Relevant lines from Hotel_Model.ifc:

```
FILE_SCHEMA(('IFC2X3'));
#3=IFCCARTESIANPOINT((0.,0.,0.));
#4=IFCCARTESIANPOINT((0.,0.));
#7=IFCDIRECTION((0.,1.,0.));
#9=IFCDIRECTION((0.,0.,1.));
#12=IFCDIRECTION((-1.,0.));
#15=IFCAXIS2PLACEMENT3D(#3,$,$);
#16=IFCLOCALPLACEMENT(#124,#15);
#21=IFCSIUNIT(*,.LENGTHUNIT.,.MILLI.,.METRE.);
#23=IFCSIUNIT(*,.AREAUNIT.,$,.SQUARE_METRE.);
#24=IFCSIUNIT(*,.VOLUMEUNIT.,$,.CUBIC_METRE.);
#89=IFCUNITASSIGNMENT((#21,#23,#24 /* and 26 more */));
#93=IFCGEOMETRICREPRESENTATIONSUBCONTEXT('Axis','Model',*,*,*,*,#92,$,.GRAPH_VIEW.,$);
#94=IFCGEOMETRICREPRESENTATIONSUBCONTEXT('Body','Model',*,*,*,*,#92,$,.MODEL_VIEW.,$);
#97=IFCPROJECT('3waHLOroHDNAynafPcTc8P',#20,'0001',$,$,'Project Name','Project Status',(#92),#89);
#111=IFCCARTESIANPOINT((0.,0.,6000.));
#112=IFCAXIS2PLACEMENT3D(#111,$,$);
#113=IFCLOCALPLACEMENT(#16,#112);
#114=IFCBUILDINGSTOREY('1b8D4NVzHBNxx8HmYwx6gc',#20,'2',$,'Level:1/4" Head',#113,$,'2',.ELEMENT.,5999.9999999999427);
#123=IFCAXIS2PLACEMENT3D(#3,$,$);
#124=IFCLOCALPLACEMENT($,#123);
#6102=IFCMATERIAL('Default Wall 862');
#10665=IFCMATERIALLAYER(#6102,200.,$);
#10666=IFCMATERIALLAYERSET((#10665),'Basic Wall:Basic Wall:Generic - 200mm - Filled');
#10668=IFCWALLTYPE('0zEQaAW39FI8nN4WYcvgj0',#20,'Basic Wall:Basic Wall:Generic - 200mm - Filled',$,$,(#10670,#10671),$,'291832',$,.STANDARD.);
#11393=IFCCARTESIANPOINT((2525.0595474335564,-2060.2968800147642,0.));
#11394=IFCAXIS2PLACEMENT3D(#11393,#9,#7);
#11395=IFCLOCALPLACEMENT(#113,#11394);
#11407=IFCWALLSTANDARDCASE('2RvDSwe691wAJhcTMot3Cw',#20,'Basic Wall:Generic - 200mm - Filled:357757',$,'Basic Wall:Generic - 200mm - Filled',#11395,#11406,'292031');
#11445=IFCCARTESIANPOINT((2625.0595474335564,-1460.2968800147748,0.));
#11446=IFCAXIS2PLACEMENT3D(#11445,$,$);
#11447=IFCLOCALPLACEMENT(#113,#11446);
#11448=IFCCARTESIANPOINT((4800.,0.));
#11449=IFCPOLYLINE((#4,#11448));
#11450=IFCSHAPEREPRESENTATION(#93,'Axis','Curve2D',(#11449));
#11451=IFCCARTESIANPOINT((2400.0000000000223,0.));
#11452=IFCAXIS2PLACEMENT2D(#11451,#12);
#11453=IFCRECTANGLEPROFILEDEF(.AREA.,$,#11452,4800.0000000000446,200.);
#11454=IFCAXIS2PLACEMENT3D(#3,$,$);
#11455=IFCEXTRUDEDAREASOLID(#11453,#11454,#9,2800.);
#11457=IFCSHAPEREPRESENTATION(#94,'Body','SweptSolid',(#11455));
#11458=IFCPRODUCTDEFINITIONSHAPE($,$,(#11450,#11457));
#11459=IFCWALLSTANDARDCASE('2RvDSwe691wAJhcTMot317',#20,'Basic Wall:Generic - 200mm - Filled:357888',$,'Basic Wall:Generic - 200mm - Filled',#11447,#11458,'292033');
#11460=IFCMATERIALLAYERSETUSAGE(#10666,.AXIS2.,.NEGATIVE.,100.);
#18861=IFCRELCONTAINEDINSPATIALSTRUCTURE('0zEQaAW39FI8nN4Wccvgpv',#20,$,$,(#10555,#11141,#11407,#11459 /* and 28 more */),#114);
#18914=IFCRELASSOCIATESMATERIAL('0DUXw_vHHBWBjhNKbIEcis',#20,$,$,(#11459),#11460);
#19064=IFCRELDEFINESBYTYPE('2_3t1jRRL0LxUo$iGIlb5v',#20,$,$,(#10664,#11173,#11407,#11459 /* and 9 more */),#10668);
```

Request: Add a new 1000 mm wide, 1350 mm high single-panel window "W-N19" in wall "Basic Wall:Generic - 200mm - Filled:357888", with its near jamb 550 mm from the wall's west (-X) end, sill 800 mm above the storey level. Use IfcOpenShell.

```python
import numpy as np
import ifcopenshell
import ifcopenshell.api.feature
import ifcopenshell.api.geometry
import ifcopenshell.api.root
import ifcopenshell.api.spatial
import ifcopenshell.api.type
import ifcopenshell.geom
import ifcopenshell.util.element
import ifcopenshell.util.placement
import ifcopenshell.util.representation
import ifcopenshell.util.shape
import ifcopenshell.util.unit

model = ifcopenshell.open("Hotel_Model.ifc")
unit_scale = ifcopenshell.util.unit.calculate_unit_scale(model)
settings = ifcopenshell.geom.settings()


def volume(element):
    """Net volume in cubic metres, openings subtracted."""
    shape = ifcopenshell.geom.create_shape(settings, element)
    return ifcopenshell.util.shape.get_volume(shape.geometry)


wall = model.by_id(11459)
storey = ifcopenshell.util.element.get_container(wall, ifc_class="IfcBuildingStorey")
context = ifcopenshell.util.representation.get_context(model, "Model", "Body", "MODEL_VIEW")
before = volume(wall)

width, height, from_end, sill = 1, 1.35, 0.55, 0.8  # metres

# The wall runs along its own X axis, and the end named is its -X end.
wall_shape = ifcopenshell.geom.create_shape(settings, wall)
x, y, z = ifcopenshell.util.shape.get_vertices(wall_shape.geometry).T
start = x.min() + from_end
face, thickness = float(y.min()), float(y.max() - y.min())
wall_matrix = ifcopenshell.util.placement.get_local_placement(wall.ObjectPlacement)
level = ifcopenshell.util.placement.get_local_placement(storey.ObjectPlacement)[2, 3]


def in_wall(x, y):
    """Placement at x, y metres in the wall's axes, at sill height."""
    matrix = wall_matrix.copy()
    matrix[:, 3] = wall_matrix @ np.array([x / unit_scale, y / unit_scale, 0.0, 1.0])
    matrix[2, 3] = level + sill / unit_scale
    return matrix


# Opening: a box that overshoots both wall faces by 50 mm.
opening = ifcopenshell.api.root.create_entity(model, ifc_class="IfcOpeningElement")
box = ifcopenshell.api.geometry.add_wall_representation(
    model, context=context, length=width, height=height, thickness=thickness + 0.1
)
ifcopenshell.api.geometry.assign_representation(model, product=opening, representation=box)
ifcopenshell.api.geometry.edit_object_placement(model, product=opening, matrix=in_wall(start, face - 0.05), is_si=False)
ifcopenshell.api.feature.add_feature(model, feature=opening, element=wall)

window = ifcopenshell.api.root.create_entity(model, ifc_class="IfcWindow", name="W-N19")
window.OverallWidth, window.OverallHeight = width / unit_scale, height / unit_scale
body = ifcopenshell.api.geometry.add_window_representation(
    model,
    context=context,
    overall_width=window.OverallWidth,
    overall_height=window.OverallHeight,
    partition_type="SINGLE_PANEL",
)
ifcopenshell.api.geometry.assign_representation(model, product=window, representation=body)
ifcopenshell.api.spatial.assign_container(model, products=[window], relating_structure=storey)
fills = ifcopenshell.api.feature.add_filling(model, opening=opening, element=window)
fills.OwnerHistory = window.OwnerHistory  # required in IFC2X3

# IFC2X3 keeps the operation on the window style.
style = ifcopenshell.api.root.create_entity(model, ifc_class="IfcWindowStyle", name="W-N19")
style.OperationType, style.ConstructionType = "SINGLE_PANEL", "NOTDEFINED"
style.ParameterTakesPrecedence = style.Sizeable = False
ifcopenshell.api.type.assign_type(model, related_objects=[window], relating_type=style)

# Centre the window in the wall's thickness.
ifcopenshell.api.geometry.edit_object_placement(model, product=window, matrix=in_wall(start, face), is_si=False)
window_shape = ifcopenshell.geom.create_shape(settings, window)
depth = ifcopenshell.util.shape.get_vertices(window_shape.geometry)[:, 1]
offset = face + thickness / 2 - (depth.min() + depth.max()) / 2
ifcopenshell.api.geometry.edit_object_placement(model, product=window, matrix=in_wall(start, offset), is_si=False)

after = volume(wall)

print(f"wall volume {before:.3f} -> {after:.3f} m3")

model.write("Hotel_Model-out.ifc")
```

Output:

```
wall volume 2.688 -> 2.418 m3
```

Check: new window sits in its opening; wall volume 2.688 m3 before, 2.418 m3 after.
